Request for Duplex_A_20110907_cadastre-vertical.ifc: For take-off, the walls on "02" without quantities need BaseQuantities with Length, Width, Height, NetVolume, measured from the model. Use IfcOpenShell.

First a look at what the model holds.

```python
import ifcopenshell
import ifcopenshell.util.element
import ifcopenshell.util.unit

model = ifcopenshell.open("Duplex_A_20110907_cadastre-vertical.ifc")
print(model.schema)
for unit_type in ("LENGTHUNIT", "AREAUNIT", "VOLUMEUNIT"):
    print(unit_type, ifcopenshell.util.unit.calculate_unit_scale(model, unit_type))
storey = next(s for s in model.by_type("IfcBuildingStorey") if s.Name == "02")
walls = [e for e in ifcopenshell.util.element.get_decomposition(storey) if e.is_a("IfcWall")]
for e in sorted(walls, key=lambda e: e.id()):
    print(e.id(), e.is_a(), e.Name, list(ifcopenshell.util.element.get_psets(e, qtos_only=True)), sep=" | ")
```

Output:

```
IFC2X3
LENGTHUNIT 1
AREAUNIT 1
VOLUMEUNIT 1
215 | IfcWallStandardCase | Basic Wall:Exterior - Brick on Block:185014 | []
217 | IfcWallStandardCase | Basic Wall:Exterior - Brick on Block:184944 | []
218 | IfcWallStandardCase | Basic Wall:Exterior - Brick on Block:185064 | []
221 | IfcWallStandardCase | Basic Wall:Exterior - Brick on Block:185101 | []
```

```python
import ifcopenshell
import ifcopenshell.api.pset
import ifcopenshell.geom
import ifcopenshell.util.element
import ifcopenshell.util.shape
import ifcopenshell.util.unit

model = ifcopenshell.open("Duplex_A_20110907_cadastre-vertical.ifc")
unit_scale = ifcopenshell.util.unit.calculate_unit_scale(model)
volume_scale = ifcopenshell.util.unit.calculate_unit_scale(model, "VOLUMEUNIT")
settings = ifcopenshell.geom.settings()

storey = next(s for s in model.by_type("IfcBuildingStorey") if s.Name == "02")
walls = [e for e in ifcopenshell.util.element.get_decomposition(storey) if e.is_a("IfcWall")]

for e in sorted(walls, key=lambda e: e.id()):
    if ifcopenshell.util.element.get_psets(e, qtos_only=True, should_inherit=False):
        continue
    # Geometry comes back in metres, in the element's own axes.
    shape = ifcopenshell.geom.create_shape(settings, e)
    values = {
        "Length": ifcopenshell.util.shape.get_x(shape.geometry) / unit_scale,
        "Width": ifcopenshell.util.shape.get_y(shape.geometry) / unit_scale,
        "Height": ifcopenshell.util.shape.get_z(shape.geometry) / unit_scale,
        "NetVolume": ifcopenshell.util.shape.get_volume(shape.geometry) / volume_scale,
    }
    qto = ifcopenshell.api.pset.add_qto(model, product=e, name="BaseQuantities")
    ifcopenshell.api.pset.edit_qto(model, qto=qto, properties=values)
    print(e.id(), {k: round(v, 3) for k, v in values.items()})

model.write("Duplex_A_20110907_cadastre-vertical_v2.ifc")
```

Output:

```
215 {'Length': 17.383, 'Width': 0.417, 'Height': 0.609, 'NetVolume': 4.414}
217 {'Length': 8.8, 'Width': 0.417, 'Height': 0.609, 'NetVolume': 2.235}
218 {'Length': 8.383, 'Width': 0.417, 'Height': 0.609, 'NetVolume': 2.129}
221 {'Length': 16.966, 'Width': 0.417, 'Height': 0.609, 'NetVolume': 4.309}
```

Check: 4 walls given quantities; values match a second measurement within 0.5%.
